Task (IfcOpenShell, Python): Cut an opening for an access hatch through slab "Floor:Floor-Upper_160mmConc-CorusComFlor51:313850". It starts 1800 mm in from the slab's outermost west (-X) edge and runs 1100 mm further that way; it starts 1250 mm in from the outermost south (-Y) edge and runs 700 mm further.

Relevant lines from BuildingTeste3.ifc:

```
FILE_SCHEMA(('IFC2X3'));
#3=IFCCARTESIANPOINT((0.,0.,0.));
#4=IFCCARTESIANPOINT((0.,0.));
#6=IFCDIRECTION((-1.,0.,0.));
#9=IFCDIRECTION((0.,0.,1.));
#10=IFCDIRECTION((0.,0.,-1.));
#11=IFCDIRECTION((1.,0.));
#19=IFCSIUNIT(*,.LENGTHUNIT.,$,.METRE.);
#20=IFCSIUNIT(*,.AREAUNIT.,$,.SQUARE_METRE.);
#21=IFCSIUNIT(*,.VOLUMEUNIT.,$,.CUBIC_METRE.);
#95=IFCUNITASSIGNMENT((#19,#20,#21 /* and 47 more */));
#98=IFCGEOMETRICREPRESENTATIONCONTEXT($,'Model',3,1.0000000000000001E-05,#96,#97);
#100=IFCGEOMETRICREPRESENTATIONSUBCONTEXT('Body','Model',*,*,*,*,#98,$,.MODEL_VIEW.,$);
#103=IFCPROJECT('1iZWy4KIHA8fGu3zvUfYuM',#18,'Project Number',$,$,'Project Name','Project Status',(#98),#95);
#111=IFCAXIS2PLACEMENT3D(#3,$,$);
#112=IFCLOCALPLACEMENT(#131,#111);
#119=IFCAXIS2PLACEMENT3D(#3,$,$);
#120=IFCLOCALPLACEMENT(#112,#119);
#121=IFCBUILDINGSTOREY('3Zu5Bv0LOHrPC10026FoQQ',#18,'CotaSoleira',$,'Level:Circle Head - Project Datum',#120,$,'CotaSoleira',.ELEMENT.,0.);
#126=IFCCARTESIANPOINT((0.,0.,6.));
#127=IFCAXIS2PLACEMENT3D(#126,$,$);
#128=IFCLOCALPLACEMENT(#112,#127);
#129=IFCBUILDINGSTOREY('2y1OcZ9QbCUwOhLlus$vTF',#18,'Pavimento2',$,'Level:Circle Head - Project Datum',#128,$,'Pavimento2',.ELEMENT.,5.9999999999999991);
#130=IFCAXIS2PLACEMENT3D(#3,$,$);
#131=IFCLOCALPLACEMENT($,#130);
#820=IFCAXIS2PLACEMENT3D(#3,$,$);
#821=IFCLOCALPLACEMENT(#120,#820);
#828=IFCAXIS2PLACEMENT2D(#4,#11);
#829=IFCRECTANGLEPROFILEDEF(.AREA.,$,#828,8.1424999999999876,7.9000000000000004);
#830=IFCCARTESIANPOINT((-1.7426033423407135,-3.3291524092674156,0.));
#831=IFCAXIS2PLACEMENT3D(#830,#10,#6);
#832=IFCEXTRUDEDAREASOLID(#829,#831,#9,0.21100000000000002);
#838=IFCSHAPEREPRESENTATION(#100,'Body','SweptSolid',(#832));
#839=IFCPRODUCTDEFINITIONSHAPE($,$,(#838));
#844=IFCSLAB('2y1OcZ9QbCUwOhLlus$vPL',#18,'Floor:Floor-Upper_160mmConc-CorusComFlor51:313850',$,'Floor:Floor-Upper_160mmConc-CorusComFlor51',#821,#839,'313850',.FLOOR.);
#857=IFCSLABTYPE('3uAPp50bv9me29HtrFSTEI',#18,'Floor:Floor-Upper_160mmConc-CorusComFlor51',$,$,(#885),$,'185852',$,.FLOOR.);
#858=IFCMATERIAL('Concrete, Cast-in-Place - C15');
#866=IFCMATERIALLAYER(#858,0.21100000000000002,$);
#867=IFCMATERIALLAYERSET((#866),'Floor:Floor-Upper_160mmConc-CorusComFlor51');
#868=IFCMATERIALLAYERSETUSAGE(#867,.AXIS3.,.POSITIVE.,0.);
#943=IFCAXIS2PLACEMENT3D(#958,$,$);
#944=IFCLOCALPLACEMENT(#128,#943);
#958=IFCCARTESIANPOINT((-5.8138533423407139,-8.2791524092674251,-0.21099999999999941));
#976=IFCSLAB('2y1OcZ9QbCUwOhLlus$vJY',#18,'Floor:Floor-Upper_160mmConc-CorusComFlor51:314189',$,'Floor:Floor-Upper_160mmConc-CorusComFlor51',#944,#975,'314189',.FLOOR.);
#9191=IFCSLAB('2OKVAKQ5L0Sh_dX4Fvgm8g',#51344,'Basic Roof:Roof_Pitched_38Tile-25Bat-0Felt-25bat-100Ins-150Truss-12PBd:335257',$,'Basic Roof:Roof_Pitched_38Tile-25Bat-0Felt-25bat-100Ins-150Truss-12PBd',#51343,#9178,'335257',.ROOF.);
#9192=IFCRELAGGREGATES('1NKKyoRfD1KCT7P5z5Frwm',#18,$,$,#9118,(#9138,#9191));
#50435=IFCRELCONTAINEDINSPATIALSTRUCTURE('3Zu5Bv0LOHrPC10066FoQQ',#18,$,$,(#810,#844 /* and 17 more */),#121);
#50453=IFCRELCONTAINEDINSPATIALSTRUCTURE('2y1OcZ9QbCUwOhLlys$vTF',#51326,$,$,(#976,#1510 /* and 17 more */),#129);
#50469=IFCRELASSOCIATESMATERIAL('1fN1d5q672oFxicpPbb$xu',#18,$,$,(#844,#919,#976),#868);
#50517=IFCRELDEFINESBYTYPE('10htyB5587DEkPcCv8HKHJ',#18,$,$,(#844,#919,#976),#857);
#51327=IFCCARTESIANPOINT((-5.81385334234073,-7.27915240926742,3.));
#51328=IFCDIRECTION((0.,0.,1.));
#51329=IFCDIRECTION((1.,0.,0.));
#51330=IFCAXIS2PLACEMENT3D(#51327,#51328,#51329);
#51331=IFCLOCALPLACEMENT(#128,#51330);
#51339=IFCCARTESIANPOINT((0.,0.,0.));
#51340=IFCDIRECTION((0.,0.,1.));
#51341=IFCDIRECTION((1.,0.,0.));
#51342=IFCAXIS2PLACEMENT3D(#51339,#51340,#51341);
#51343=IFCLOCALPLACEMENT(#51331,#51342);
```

```python
import numpy as np
import ifcopenshell
import ifcopenshell.api.feature
import ifcopenshell.api.geometry
import ifcopenshell.api.root
import ifcopenshell.geom
import ifcopenshell.util.placement
import ifcopenshell.util.representation
import ifcopenshell.util.shape
import ifcopenshell.util.unit

model = ifcopenshell.open("BuildingTeste3.ifc")
unit_scale = ifcopenshell.util.unit.calculate_unit_scale(model)
settings = ifcopenshell.geom.settings()


def volume(element):
    """Net volume in cubic metres, openings subtracted."""
    shape = ifcopenshell.geom.create_shape(settings, element)
    return ifcopenshell.util.shape.get_volume(shape.geometry)


slab = model.by_guid("2y1OcZ9QbCUwOhLlus$vPL")
before = volume(slab)

# Extent in the slab's own axes, in metres. The edges named are its -X and -Y sides.
slab_shape = ifcopenshell.geom.create_shape(settings, slab)
vertices = ifcopenshell.util.shape.get_vertices(slab_shape.geometry)
x_min, y_min, bottom = vertices.min(axis=0)
top = vertices[:, 2].max()

opening = ifcopenshell.api.root.create_entity(model, ifc_class="IfcOpeningElement", name="Access hatch opening")
context = ifcopenshell.util.representation.get_context(model, "Model", "Body", "MODEL_VIEW")
width, depth = 1.1, 0.7
outline = [(0.0, 0.0), (width, 0.0), (width, depth), (0.0, depth), (0.0, 0.0)]
# Overshoot both faces by 50 mm so the cut is clean.
shape = ifcopenshell.api.geometry.add_slab_representation(
    model, context=context, depth=top - bottom + 0.1, polyline=outline
)
ifcopenshell.api.geometry.assign_representation(model, product=opening, representation=shape)

matrix = ifcopenshell.util.placement.get_local_placement(slab.ObjectPlacement)
matrix[:, 3] = matrix @ np.append(np.array([x_min + 1.8, y_min + 1.25, bottom - 0.05]) / unit_scale, 1.0)
ifcopenshell.api.geometry.edit_object_placement(model, product=opening, matrix=matrix, is_si=False)
ifcopenshell.api.feature.add_feature(model, feature=opening, element=slab)

after = volume(slab)

print(f"slab volume {before:.3f} -> {after:.3f} m3")

model.write("BuildingTeste3_rev.ifc")
```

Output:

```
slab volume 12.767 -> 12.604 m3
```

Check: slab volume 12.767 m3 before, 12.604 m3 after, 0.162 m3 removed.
